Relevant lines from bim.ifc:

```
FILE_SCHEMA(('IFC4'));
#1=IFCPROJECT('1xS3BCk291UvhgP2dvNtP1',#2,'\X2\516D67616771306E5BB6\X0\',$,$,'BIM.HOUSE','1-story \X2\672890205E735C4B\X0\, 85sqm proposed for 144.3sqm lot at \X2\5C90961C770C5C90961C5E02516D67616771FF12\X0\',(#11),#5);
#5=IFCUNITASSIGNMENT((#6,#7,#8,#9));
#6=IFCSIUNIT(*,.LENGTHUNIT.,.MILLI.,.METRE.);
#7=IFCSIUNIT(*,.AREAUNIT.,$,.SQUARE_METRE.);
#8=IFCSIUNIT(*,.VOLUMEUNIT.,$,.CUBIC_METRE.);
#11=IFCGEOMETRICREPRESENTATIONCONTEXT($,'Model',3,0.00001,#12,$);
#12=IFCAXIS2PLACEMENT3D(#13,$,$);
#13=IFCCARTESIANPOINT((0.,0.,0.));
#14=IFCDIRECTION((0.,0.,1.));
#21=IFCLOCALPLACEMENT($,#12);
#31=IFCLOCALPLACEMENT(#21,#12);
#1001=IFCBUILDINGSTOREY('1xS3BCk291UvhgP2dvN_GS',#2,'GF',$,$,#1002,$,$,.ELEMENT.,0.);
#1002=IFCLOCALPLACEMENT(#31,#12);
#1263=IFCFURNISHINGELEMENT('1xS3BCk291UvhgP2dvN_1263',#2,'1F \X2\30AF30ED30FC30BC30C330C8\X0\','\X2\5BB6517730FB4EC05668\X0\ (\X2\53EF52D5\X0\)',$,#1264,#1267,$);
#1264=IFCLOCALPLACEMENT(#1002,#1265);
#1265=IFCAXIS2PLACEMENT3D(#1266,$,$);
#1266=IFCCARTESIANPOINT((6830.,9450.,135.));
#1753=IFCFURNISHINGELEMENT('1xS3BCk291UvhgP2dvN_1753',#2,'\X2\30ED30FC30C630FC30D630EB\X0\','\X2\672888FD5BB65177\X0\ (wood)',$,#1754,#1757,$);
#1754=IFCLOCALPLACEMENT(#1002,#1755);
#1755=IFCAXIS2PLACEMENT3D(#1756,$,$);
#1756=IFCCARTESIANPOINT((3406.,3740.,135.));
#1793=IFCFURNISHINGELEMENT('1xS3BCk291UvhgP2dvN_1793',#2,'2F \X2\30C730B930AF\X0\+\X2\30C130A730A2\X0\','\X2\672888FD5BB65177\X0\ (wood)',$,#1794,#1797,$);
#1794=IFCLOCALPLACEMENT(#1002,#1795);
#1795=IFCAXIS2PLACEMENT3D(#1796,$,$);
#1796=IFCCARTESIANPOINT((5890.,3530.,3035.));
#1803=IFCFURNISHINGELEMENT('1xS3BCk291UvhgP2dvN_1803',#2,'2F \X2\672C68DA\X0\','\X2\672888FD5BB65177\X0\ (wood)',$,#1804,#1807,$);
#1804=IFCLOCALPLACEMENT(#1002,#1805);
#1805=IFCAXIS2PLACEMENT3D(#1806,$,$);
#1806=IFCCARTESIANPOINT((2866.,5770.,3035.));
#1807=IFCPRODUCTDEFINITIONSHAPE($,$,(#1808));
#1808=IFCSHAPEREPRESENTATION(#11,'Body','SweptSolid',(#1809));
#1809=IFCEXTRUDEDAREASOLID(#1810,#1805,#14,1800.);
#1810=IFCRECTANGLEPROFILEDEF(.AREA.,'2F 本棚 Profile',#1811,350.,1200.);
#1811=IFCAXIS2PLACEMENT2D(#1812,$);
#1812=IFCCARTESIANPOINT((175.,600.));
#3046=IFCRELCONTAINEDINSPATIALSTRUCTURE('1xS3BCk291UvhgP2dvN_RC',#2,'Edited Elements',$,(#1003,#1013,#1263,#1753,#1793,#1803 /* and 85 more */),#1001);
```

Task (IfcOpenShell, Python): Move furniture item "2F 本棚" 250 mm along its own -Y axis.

```python
import ifcopenshell
import ifcopenshell.api.geometry
import ifcopenshell.util.placement
import ifcopenshell.util.unit

model = ifcopenshell.open("bim.ifc")
unit_scale = ifcopenshell.util.unit.calculate_unit_scale(model)

item = model.by_guid("1xS3BCk291UvhgP2dvN_1803")
matrix = ifcopenshell.util.placement.get_local_placement(item.ObjectPlacement)
matrix[:3, 3] -= matrix[:3, 1] * 0.25 / unit_scale
ifcopenshell.api.geometry.edit_object_placement(model, product=item, matrix=matrix, is_si=False)

print(ifcopenshell.util.placement.get_local_placement(item.ObjectPlacement).round(3) + 0.0)

model.write("bim-out.ifc")
```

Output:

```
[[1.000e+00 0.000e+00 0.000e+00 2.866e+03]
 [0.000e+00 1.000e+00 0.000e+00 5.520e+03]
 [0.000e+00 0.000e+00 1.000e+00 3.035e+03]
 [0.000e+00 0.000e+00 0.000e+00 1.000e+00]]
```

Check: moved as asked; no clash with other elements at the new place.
